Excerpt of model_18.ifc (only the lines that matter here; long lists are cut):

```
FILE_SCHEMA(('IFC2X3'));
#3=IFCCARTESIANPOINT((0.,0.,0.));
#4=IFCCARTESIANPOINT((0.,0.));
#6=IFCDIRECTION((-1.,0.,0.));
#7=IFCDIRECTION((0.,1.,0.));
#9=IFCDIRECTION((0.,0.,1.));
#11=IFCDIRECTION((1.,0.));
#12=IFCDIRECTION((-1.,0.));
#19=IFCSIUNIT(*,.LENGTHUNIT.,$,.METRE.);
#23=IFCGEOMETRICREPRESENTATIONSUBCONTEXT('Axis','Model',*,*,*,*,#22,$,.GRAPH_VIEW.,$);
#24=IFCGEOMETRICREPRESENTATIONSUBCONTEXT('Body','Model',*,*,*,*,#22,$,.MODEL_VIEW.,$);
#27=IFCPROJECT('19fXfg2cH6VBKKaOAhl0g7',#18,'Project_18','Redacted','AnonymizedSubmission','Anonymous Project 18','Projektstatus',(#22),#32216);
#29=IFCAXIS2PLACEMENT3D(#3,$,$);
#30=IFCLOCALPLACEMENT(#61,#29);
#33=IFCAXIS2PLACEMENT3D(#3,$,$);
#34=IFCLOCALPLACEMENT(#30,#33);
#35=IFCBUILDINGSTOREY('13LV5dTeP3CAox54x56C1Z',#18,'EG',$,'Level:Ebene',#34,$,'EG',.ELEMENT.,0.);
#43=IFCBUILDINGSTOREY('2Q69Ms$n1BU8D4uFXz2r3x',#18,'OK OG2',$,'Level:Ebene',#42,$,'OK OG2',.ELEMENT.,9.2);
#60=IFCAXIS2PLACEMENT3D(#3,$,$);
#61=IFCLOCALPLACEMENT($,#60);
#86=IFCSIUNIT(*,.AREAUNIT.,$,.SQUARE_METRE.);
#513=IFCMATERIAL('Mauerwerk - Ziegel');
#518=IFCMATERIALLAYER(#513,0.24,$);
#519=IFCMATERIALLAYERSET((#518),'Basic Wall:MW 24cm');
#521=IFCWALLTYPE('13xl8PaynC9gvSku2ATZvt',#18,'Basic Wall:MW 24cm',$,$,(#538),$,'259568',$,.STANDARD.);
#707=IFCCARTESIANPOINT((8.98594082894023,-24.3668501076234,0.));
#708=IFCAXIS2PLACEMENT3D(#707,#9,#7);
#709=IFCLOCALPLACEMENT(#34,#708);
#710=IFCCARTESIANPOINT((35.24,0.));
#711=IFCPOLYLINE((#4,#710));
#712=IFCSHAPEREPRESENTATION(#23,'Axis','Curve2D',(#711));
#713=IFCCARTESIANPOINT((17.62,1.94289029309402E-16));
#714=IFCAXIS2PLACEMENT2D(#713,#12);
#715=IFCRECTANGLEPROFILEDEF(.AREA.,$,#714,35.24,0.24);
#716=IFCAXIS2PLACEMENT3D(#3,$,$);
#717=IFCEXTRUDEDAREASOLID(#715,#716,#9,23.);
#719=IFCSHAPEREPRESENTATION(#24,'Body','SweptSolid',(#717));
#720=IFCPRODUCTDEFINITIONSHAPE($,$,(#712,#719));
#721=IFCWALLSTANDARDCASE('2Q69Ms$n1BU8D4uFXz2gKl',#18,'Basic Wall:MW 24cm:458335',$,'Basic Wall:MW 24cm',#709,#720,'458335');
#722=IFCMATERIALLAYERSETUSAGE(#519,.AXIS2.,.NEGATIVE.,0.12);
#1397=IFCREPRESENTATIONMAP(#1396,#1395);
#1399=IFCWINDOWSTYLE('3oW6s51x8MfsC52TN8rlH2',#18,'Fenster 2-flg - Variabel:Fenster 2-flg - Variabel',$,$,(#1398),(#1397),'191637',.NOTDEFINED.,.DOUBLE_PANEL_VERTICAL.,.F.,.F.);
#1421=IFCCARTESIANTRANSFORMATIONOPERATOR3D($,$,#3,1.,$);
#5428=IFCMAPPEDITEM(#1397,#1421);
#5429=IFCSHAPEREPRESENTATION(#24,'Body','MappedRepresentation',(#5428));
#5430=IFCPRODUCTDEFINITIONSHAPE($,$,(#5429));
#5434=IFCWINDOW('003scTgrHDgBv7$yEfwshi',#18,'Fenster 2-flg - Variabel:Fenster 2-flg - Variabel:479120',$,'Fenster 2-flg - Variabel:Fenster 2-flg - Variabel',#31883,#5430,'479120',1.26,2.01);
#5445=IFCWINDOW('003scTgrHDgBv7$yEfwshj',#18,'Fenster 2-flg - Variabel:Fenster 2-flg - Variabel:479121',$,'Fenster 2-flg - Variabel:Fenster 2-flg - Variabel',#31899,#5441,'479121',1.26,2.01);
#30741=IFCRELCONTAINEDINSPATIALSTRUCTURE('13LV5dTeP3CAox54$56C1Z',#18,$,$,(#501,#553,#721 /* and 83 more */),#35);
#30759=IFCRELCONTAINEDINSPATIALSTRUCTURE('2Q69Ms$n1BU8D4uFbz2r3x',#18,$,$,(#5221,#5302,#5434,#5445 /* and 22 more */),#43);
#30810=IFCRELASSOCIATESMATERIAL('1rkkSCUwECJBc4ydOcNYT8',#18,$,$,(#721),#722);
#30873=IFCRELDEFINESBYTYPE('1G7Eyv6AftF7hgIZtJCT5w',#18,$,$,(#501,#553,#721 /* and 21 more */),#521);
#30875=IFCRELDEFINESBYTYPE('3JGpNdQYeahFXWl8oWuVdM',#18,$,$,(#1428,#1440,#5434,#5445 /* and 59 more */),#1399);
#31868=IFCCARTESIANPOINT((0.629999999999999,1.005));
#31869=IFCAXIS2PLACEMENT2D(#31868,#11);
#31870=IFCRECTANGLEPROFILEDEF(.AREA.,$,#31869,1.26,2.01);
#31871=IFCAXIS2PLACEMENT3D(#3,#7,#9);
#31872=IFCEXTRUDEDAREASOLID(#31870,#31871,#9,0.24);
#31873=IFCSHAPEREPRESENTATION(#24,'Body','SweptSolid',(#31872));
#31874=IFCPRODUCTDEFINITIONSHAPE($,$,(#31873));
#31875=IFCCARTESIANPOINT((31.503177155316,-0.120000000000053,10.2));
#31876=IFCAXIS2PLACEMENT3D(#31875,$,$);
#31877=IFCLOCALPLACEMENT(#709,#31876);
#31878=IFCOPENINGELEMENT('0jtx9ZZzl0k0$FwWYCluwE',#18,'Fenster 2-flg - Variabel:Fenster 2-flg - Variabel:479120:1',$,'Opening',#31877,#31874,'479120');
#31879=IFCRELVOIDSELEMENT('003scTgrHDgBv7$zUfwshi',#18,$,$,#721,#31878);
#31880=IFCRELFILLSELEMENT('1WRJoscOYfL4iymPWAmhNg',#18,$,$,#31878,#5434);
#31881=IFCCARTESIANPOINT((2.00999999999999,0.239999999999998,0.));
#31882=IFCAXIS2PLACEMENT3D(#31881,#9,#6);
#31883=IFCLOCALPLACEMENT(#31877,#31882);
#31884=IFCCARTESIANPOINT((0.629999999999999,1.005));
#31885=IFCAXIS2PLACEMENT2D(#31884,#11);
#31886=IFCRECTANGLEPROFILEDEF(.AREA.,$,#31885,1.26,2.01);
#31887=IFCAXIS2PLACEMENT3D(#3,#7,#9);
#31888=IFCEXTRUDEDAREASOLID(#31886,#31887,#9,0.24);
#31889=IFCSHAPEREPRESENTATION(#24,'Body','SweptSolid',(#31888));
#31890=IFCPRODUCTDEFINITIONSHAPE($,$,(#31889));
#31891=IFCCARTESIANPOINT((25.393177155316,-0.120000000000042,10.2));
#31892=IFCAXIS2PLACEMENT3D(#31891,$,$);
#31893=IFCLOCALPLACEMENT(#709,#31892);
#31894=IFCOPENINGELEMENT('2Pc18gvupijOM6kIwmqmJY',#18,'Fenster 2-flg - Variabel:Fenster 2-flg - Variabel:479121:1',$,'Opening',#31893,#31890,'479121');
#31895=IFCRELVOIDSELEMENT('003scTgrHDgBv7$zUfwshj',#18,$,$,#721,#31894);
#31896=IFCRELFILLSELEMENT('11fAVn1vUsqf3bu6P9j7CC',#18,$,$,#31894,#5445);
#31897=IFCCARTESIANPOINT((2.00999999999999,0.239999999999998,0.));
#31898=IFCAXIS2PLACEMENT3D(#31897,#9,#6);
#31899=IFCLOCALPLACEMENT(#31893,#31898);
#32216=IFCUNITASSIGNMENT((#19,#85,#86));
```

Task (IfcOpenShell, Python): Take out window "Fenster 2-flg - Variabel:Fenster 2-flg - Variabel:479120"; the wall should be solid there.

```python
import ifcopenshell
import ifcopenshell.api.feature
import ifcopenshell.api.root
import ifcopenshell.geom
import ifcopenshell.util.shape

model = ifcopenshell.open("model_18.ifc")
settings = ifcopenshell.geom.settings()


def volume(element):
    """Net volume in cubic metres, openings subtracted."""
    shape = ifcopenshell.geom.create_shape(settings, element)
    return ifcopenshell.util.shape.get_volume(shape.geometry)


window = model.by_id(5434)
opening = window.FillsVoids[0].RelatingOpeningElement
wall = opening.VoidsElements[0].RelatingBuildingElement
before = volume(wall)

ifcopenshell.api.root.remove_product(model, product=window)
ifcopenshell.api.feature.remove_feature(model, feature=opening)

after = volume(wall)

print(f"wall volume {before:.3f} -> {after:.3f} m3")

model.write("model_18_rev.ifc")
```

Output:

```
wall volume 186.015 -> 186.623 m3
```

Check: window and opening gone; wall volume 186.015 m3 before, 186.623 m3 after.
